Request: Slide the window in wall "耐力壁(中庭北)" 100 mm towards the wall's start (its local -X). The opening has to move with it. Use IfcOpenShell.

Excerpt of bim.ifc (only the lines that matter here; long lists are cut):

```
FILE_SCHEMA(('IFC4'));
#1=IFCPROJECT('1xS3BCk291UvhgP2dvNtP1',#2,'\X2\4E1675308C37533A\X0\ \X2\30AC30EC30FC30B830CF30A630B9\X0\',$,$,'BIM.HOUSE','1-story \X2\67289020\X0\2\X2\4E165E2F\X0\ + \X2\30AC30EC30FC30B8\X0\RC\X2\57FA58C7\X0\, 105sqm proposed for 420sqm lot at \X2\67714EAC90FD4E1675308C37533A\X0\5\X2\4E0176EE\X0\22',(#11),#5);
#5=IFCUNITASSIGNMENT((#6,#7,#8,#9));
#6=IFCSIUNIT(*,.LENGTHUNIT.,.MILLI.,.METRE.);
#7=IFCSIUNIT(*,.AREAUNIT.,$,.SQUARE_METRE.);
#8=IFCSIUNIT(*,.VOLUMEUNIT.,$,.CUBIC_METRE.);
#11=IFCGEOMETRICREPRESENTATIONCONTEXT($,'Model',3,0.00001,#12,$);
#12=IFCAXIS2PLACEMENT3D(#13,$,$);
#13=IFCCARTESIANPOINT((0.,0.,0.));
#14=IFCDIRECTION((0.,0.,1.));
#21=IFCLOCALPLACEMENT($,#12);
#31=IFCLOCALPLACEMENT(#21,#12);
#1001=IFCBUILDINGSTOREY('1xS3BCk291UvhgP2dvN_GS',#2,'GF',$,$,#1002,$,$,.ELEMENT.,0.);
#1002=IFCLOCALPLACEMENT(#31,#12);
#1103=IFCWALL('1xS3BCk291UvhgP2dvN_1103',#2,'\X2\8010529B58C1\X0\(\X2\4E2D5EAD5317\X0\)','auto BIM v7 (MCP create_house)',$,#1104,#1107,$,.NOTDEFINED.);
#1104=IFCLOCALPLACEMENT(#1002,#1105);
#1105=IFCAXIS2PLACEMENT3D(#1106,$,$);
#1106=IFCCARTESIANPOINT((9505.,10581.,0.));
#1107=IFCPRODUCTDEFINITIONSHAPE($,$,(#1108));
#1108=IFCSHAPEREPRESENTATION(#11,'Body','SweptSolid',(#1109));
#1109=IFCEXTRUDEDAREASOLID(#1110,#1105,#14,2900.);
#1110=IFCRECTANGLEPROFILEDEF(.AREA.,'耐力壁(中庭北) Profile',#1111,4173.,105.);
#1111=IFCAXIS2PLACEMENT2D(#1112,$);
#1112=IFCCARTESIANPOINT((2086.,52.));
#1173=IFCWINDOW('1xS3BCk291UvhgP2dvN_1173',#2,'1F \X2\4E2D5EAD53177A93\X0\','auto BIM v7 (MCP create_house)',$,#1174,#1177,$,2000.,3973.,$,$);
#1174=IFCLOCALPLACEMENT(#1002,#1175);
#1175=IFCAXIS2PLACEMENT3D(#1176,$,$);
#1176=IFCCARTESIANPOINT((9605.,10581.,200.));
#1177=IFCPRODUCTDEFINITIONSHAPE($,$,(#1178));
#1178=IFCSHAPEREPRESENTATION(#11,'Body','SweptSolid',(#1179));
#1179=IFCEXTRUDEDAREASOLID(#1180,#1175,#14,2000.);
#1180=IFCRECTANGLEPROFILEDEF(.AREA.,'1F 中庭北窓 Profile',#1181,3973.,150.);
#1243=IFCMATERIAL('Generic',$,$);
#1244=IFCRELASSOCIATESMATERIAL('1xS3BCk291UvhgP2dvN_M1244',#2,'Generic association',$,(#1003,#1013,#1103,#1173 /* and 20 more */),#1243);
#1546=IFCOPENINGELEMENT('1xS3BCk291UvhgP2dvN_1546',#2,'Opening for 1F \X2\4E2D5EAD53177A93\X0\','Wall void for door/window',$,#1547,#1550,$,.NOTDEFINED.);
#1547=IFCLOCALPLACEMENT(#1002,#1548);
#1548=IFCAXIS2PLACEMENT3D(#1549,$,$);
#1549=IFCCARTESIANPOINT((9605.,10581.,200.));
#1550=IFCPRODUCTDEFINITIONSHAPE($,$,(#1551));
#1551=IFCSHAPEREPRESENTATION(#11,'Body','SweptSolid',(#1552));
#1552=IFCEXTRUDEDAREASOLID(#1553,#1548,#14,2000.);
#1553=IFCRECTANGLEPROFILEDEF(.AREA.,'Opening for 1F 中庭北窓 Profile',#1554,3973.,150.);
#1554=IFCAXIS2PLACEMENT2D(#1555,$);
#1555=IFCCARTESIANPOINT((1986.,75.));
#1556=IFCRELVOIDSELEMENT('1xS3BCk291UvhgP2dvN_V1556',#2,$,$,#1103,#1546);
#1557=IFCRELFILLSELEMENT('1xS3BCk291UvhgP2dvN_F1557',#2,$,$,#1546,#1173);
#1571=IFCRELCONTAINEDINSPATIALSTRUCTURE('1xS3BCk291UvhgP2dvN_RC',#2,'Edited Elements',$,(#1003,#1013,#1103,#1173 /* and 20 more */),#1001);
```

```python
import ifcopenshell
import ifcopenshell.api.geometry
import ifcopenshell.util.placement

model = ifcopenshell.open("bim.ifc")

window = model.by_guid("1xS3BCk291UvhgP2dvN_1173")
opening = window.FillsVoids[0].RelatingOpeningElement
wall = opening.VoidsElements[0].RelatingBuildingElement

wall_matrix = ifcopenshell.util.placement.get_local_placement(wall.ObjectPlacement)
shift = wall_matrix[:3, 0] * -100.0
before = ifcopenshell.util.placement.get_local_placement(window.ObjectPlacement)[:3, 3].copy()

# The window is not placed relative to its opening, so move both.
for product in (opening, window):
    matrix = ifcopenshell.util.placement.get_local_placement(product.ObjectPlacement)
    matrix[:3, 3] += shift
    ifcopenshell.api.geometry.edit_object_placement(model, product=product, matrix=matrix, is_si=False)

after = ifcopenshell.util.placement.get_local_placement(window.ObjectPlacement)[:3, 3]
print("window moved by", (after - before).round(3) + 0.0)

model.write("bim_edited.ifc")
```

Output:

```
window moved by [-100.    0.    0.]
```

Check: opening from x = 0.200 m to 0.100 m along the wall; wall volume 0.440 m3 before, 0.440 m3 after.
